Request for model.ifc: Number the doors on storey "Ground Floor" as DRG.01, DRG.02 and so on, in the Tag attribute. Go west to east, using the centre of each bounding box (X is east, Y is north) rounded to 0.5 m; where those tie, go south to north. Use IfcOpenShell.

First a look at what the model holds.

```python
import ifcopenshell
import ifcopenshell.util.element
import ifcopenshell.util.placement

model = ifcopenshell.open("model.ifc")
print(model.schema)
storey = next(s for s in model.by_type("IfcBuildingStorey") if s.Name == "Ground Floor")
doors = [e for e in ifcopenshell.util.element.get_decomposition(storey) if e.is_a("IfcDoor")]
for e in sorted(doors, key=lambda e: e.id()):
    origin = ifcopenshell.util.placement.get_local_placement(e.ObjectPlacement)[:3, 3]
    print(e.id(), e.Tag, e.Name, origin.round(2) + 0.0, sep=" | ")
```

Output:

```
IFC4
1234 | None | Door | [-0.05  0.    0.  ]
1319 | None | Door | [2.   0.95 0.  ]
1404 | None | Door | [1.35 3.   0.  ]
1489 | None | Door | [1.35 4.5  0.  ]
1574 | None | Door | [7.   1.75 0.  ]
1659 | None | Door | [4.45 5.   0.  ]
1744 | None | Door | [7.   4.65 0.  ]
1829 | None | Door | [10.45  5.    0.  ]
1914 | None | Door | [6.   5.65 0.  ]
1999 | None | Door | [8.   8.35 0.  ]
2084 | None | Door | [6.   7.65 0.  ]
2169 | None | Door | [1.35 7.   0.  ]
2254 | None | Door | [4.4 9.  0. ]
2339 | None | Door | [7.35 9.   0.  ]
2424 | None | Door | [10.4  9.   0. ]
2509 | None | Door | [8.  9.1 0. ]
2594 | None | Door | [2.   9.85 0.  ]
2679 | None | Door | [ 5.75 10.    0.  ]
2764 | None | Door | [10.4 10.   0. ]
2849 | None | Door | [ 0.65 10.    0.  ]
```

```python
import ifcopenshell
import ifcopenshell.geom
import ifcopenshell.util.element
import ifcopenshell.util.shape

model = ifcopenshell.open("model.ifc")
settings = ifcopenshell.geom.settings()
settings.set("use-world-coords", True)


def centre(element):
    shape = ifcopenshell.geom.create_shape(settings, element)
    return ifcopenshell.util.shape.get_bbox_centroid(shape.geometry)


storey = next(s for s in model.by_type("IfcBuildingStorey") if s.Name == "Ground Floor")
doors = [e for e in ifcopenshell.util.element.get_decomposition(storey) if e.is_a("IfcDoor")]

# Insertion points can sit at a corner or the storey origin, so sort by the geometry (in metres).
centres = {e: centre(e) for e in doors}
doors.sort(key=lambda e: (round(centres[e][0] / 0.5), centres[e][1]))

for i, e in enumerate(doors, start=1):
    number = f"DRG.{i:02d}"
    e.Tag = number
    print(e.id(), number)

model.write("model-out.ifc")
```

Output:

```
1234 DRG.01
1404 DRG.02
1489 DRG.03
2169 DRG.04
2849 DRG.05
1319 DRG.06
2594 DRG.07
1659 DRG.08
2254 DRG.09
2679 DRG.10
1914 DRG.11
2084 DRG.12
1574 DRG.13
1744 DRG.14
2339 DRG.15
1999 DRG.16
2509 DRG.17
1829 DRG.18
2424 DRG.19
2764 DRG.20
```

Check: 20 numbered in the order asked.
